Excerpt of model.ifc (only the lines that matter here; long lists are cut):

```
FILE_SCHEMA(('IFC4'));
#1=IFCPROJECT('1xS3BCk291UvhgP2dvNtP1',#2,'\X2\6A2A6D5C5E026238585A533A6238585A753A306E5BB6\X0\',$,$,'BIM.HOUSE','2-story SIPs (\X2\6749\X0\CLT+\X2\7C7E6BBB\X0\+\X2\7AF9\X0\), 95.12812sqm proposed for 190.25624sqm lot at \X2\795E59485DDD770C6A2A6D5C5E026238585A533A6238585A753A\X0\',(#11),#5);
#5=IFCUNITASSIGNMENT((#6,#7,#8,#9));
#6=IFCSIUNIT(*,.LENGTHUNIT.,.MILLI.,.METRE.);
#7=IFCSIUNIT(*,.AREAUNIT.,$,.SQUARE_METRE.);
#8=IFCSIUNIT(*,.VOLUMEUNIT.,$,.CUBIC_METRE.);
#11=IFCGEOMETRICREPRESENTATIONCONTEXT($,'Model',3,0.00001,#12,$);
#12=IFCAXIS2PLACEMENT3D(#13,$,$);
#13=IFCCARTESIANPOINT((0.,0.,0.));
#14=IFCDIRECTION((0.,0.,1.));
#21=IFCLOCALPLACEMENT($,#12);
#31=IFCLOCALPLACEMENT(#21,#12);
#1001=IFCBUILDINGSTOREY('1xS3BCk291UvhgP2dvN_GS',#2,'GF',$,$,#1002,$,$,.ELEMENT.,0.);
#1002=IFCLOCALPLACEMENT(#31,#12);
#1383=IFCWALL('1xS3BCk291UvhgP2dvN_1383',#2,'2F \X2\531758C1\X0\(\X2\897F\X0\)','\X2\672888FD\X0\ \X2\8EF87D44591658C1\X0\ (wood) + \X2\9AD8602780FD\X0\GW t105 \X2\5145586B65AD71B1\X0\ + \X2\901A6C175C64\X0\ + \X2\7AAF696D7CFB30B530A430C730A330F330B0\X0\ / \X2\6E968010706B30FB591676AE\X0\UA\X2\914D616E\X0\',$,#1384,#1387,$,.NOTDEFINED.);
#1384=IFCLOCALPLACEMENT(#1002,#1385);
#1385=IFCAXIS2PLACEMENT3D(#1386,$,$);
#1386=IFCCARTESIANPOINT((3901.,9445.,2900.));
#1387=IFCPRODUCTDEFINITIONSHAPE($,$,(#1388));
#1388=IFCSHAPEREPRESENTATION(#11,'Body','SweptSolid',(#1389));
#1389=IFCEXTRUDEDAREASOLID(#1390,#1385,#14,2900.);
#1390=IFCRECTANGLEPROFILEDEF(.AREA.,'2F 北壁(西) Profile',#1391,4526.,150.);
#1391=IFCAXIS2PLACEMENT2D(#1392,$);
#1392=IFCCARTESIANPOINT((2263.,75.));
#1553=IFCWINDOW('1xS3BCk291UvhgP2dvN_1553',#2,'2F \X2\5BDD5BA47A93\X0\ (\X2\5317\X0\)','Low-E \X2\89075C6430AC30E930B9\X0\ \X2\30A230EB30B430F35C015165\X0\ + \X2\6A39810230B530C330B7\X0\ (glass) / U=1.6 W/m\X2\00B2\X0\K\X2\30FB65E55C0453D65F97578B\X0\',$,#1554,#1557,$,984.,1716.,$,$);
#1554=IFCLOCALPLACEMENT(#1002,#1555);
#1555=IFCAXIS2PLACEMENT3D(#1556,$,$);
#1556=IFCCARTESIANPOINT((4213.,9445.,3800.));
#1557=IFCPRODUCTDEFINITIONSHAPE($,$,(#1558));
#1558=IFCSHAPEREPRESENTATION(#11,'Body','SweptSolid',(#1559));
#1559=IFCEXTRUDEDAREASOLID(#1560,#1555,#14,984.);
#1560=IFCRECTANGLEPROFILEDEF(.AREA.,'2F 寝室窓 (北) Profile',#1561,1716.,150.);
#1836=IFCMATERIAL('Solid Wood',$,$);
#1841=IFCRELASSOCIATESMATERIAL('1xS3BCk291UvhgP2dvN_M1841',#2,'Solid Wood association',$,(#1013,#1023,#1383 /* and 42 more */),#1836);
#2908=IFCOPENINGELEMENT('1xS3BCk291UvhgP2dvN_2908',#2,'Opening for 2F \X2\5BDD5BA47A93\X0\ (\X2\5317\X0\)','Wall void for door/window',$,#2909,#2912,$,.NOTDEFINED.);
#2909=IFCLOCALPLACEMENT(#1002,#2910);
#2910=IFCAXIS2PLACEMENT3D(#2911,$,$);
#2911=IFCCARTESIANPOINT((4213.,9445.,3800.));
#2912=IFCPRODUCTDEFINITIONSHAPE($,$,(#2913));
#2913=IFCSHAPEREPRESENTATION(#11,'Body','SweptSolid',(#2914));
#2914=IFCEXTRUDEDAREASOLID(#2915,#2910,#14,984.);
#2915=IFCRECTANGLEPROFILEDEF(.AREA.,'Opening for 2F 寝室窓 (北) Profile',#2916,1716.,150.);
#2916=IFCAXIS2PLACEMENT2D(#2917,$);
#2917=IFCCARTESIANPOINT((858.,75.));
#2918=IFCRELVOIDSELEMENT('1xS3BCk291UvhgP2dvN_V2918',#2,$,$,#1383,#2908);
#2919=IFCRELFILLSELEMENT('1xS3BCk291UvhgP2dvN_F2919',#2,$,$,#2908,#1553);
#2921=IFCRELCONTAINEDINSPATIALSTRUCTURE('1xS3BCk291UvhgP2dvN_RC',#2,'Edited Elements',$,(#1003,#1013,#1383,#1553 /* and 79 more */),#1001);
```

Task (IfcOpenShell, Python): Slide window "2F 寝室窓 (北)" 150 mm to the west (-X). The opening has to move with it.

```python
import ifcopenshell
import ifcopenshell.api.geometry
import ifcopenshell.util.placement
import ifcopenshell.util.unit

model = ifcopenshell.open("model.ifc")
unit_scale = ifcopenshell.util.unit.calculate_unit_scale(model)

window = model.by_id(1553)
opening = window.FillsVoids[0].RelatingOpeningElement
wall = opening.VoidsElements[0].RelatingBuildingElement

wall_matrix = ifcopenshell.util.placement.get_local_placement(wall.ObjectPlacement)
shift = wall_matrix[:3, 0] * -0.15 / unit_scale
before = ifcopenshell.util.placement.get_local_placement(window.ObjectPlacement)[:3, 3].copy()

# The window is not placed relative to its opening, so move both.
for product in (opening, window):
    matrix = ifcopenshell.util.placement.get_local_placement(product.ObjectPlacement)
    matrix[:3, 3] += shift
    ifcopenshell.api.geometry.edit_object_placement(model, product=product, matrix=matrix, is_si=False)

after = ifcopenshell.util.placement.get_local_placement(window.ObjectPlacement)[:3, 3]
print("window moved by", (after - before).round(3) + 0.0)

model.write("model_edited.ifc")
```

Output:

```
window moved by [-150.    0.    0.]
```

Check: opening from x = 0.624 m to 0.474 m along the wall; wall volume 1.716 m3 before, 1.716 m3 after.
